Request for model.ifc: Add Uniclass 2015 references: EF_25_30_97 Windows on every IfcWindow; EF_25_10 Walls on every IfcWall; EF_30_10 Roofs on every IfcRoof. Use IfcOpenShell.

First a look at what the model holds.

```python
import ifcopenshell

model = ifcopenshell.open("model.ifc")
print(model.schema)
print("classifications:", [c.Name for c in model.by_type("IfcClassification")])
for ifc_class in ("IfcDoor", "IfcRoof", "IfcStair", "IfcWall", "IfcWindow"):
    print(ifc_class, len(model.by_type(ifc_class)))
```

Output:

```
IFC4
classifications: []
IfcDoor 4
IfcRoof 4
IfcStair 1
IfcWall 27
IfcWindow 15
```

```python
import ifcopenshell
import ifcopenshell.api.classification

model = ifcopenshell.open("model.ifc")

system = ifcopenshell.api.classification.add_classification(model, classification="Uniclass 2015")

codes = {
    "IfcWindow": ("EF_25_30_97", "Windows"),
    "IfcWall": ("EF_25_10", "Walls"),
    "IfcRoof": ("EF_30_10", "Roofs"),
}
for ifc_class, (code, name) in codes.items():
    products = model.by_type(ifc_class)
    ifcopenshell.api.classification.add_reference(
        model, products=products, classification=system, identification=code, name=name
    )
    print(code, len(products))

model.write("model-out.ifc")
```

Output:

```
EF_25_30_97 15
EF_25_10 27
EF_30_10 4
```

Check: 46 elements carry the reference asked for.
